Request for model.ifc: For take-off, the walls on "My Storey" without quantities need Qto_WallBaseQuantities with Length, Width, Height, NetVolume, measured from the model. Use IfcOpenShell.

First a look at what the model holds.

```python
import ifcopenshell
import ifcopenshell.util.element
import ifcopenshell.util.unit

model = ifcopenshell.open("model.ifc")
print(model.schema)
for unit_type in ("LENGTHUNIT", "AREAUNIT", "VOLUMEUNIT"):
    print(unit_type, ifcopenshell.util.unit.calculate_unit_scale(model, unit_type))
storey = next(s for s in model.by_type("IfcBuildingStorey") if s.Name == "My Storey")
walls = [e for e in ifcopenshell.util.element.get_decomposition(storey) if e.is_a("IfcWall")]
for e in sorted(walls, key=lambda e: e.id()):
    print(e.id(), e.is_a(), e.Name, list(ifcopenshell.util.element.get_psets(e, qtos_only=True)), sep=" | ")
```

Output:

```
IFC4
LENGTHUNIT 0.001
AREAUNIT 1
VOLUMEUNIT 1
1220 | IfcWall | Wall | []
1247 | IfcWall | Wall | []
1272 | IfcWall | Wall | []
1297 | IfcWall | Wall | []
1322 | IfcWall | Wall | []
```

```python
import ifcopenshell
import ifcopenshell.api.pset
import ifcopenshell.geom
import ifcopenshell.util.element
import ifcopenshell.util.shape
import ifcopenshell.util.unit

model = ifcopenshell.open("model.ifc")
unit_scale = ifcopenshell.util.unit.calculate_unit_scale(model)
volume_scale = ifcopenshell.util.unit.calculate_unit_scale(model, "VOLUMEUNIT")
settings = ifcopenshell.geom.settings()

storey = next(s for s in model.by_type("IfcBuildingStorey") if s.Name == "My Storey")
walls = [e for e in ifcopenshell.util.element.get_decomposition(storey) if e.is_a("IfcWall")]

for e in sorted(walls, key=lambda e: e.id()):
    if ifcopenshell.util.element.get_psets(e, qtos_only=True, should_inherit=False):
        continue
    # Geometry comes back in metres, in the element's own axes.
    shape = ifcopenshell.geom.create_shape(settings, e)
    values = {
        "Length": ifcopenshell.util.shape.get_x(shape.geometry) / unit_scale,
        "Width": ifcopenshell.util.shape.get_y(shape.geometry) / unit_scale,
        "Height": ifcopenshell.util.shape.get_z(shape.geometry) / unit_scale,
        "NetVolume": ifcopenshell.util.shape.get_volume(shape.geometry) / volume_scale,
    }
    qto = ifcopenshell.api.pset.add_qto(model, product=e, name="Qto_WallBaseQuantities")
    ifcopenshell.api.pset.edit_qto(model, qto=qto, properties=values)
    print(e.id(), {k: round(v, 3) for k, v in values.items()})

model.write("model_rev.ifc")
```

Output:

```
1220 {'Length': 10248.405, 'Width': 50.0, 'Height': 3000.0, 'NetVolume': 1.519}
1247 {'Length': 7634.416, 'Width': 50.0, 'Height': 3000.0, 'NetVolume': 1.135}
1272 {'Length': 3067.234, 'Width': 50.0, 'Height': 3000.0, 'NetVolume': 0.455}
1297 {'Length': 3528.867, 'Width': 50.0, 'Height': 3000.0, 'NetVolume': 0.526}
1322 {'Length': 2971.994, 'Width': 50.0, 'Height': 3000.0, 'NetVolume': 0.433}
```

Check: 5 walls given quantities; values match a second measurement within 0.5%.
